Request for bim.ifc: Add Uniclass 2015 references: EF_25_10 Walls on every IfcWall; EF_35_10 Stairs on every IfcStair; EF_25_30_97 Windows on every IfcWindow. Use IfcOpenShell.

First a look at what the model holds.

```python
import ifcopenshell

model = ifcopenshell.open("bim.ifc")
print(model.schema)
print("classifications:", [c.Name for c in model.by_type("IfcClassification")])
for ifc_class in ("IfcDoor", "IfcRoof", "IfcStair", "IfcWall", "IfcWindow"):
    print(ifc_class, len(model.by_type(ifc_class)))
```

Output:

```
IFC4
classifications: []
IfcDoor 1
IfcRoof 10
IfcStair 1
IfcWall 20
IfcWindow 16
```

```python
import ifcopenshell
import ifcopenshell.api.classification

model = ifcopenshell.open("bim.ifc")

system = ifcopenshell.api.classification.add_classification(model, classification="Uniclass 2015")

codes = {
    "IfcWall": ("EF_25_10", "Walls"),
    "IfcStair": ("EF_35_10", "Stairs"),
    "IfcWindow": ("EF_25_30_97", "Windows"),
}
for ifc_class, (code, name) in codes.items():
    products = model.by_type(ifc_class)
    ifcopenshell.api.classification.add_reference(
        model, products=products, classification=system, identification=code, name=name
    )
    print(code, len(products))

model.write("bim_edited.ifc")
```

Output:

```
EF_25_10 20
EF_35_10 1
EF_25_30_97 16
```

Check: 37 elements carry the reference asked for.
